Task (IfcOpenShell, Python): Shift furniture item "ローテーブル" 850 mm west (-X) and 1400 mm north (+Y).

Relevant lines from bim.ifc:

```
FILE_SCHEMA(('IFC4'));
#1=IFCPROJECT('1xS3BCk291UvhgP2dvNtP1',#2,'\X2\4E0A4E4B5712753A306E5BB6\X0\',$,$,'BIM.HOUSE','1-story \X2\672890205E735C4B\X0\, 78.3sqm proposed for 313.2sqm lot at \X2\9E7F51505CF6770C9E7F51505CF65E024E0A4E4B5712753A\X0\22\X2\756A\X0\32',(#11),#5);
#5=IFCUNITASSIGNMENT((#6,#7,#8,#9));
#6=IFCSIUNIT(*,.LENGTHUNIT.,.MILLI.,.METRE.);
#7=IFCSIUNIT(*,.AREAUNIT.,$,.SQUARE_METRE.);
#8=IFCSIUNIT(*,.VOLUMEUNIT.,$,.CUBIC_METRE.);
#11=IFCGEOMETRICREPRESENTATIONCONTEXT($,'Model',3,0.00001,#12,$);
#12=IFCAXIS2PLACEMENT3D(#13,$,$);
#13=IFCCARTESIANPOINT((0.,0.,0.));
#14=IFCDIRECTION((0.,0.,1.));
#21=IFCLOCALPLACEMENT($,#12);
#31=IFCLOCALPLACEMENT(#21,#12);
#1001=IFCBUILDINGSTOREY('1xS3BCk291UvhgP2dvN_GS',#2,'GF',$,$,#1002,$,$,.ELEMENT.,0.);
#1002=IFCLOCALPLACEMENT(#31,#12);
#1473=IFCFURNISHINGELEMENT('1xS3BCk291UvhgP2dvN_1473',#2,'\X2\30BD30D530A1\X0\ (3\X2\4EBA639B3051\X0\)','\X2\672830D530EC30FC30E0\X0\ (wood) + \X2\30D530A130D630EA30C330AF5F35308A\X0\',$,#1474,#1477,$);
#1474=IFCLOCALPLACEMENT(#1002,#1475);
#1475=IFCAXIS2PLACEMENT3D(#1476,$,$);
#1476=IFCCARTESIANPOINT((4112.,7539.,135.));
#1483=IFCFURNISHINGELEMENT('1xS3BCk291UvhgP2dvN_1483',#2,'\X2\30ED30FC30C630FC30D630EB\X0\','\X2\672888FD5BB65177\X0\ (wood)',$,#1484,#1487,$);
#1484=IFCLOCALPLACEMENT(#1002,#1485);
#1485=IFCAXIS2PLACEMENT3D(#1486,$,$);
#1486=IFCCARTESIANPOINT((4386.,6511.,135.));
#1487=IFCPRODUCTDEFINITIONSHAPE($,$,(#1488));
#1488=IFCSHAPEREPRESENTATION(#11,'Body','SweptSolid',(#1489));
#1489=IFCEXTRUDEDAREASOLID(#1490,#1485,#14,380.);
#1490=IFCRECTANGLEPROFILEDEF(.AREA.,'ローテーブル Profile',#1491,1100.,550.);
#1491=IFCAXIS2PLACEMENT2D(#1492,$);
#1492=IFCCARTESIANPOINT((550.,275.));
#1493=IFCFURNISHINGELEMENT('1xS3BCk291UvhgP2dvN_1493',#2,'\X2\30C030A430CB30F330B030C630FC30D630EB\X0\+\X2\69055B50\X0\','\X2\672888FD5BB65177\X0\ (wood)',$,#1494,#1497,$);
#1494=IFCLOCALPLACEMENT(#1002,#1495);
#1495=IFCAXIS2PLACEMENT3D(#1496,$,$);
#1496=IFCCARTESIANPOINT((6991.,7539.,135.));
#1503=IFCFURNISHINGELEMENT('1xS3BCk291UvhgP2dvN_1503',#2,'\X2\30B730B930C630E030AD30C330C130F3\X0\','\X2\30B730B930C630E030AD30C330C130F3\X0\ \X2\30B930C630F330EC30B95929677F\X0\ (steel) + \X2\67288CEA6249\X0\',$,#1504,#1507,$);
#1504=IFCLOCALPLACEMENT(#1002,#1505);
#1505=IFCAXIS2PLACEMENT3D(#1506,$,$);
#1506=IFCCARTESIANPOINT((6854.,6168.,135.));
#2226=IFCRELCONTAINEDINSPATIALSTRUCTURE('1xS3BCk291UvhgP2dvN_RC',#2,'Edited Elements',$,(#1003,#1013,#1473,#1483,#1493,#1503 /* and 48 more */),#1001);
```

```python
import ifcopenshell
import ifcopenshell.api.geometry
import ifcopenshell.util.placement
import ifcopenshell.util.unit

model = ifcopenshell.open("bim.ifc")
unit_scale = ifcopenshell.util.unit.calculate_unit_scale(model)

item = model.by_guid("1xS3BCk291UvhgP2dvN_1483")
matrix = ifcopenshell.util.placement.get_local_placement(item.ObjectPlacement)
matrix[0, 3] -= 0.85 / unit_scale
matrix[1, 3] += 1.4 / unit_scale
ifcopenshell.api.geometry.edit_object_placement(model, product=item, matrix=matrix, is_si=False)

print(ifcopenshell.util.placement.get_local_placement(item.ObjectPlacement).round(3) + 0.0)

model.write("bim_edited.ifc")
```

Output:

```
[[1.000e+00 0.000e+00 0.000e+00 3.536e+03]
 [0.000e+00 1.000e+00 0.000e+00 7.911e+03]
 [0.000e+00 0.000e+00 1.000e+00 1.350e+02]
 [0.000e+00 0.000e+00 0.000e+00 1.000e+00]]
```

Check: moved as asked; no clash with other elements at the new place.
